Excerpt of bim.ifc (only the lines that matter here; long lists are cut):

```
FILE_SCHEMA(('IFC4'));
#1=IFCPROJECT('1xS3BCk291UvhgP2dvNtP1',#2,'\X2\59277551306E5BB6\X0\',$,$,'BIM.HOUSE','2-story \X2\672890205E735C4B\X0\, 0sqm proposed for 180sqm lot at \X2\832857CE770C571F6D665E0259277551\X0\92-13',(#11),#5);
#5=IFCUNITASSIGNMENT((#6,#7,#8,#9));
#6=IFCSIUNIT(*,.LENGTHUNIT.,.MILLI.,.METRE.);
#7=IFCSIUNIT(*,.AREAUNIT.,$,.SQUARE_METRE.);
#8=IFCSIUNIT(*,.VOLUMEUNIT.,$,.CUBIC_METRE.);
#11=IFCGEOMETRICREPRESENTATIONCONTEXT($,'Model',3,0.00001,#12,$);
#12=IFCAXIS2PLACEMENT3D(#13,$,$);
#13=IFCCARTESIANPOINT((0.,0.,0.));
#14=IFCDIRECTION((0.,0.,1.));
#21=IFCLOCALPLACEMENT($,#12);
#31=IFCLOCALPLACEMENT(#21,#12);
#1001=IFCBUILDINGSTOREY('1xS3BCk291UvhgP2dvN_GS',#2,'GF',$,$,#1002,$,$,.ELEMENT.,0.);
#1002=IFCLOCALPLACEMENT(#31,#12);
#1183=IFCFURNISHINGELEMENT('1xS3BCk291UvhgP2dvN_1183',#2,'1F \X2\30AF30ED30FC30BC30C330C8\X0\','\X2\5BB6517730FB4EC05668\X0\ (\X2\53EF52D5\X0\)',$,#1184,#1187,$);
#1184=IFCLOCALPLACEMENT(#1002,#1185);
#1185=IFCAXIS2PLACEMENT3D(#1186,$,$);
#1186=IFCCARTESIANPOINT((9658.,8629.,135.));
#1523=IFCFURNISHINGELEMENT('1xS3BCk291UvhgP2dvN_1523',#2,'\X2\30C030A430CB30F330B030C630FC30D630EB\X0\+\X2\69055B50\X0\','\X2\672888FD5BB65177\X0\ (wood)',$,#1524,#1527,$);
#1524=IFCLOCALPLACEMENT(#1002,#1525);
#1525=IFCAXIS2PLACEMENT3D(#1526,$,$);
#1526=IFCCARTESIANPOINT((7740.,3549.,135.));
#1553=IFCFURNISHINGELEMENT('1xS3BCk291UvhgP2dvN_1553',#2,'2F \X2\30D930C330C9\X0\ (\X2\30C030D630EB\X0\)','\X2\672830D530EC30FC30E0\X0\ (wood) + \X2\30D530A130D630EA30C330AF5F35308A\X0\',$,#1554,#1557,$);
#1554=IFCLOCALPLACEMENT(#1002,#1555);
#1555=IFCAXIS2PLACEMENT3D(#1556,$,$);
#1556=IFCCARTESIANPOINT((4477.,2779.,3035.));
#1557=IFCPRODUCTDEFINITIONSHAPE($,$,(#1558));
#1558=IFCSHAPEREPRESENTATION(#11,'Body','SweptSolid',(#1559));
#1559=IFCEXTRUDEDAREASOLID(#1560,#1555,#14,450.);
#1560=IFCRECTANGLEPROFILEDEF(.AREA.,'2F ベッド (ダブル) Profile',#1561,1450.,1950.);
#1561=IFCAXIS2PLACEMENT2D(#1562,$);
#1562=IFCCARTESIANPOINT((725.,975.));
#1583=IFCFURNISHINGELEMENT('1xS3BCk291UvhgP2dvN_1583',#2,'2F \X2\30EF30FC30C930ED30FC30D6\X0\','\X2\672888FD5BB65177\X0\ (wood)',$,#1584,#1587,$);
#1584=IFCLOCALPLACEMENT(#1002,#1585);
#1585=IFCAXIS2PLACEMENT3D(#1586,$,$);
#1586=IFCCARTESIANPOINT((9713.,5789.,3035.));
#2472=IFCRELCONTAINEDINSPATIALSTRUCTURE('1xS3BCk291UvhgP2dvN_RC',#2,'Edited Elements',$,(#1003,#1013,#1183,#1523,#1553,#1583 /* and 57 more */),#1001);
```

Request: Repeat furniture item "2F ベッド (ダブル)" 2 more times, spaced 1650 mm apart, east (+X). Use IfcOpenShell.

```python
import numpy as np
import ifcopenshell
import ifcopenshell.api.geometry
import ifcopenshell.api.root
import ifcopenshell.util.element
import ifcopenshell.util.placement
import ifcopenshell.util.unit

model = ifcopenshell.open("bim.ifc")
unit_scale = ifcopenshell.util.unit.calculate_unit_scale(model)


def reuse_history(source, copy):
    """copy_class also copies each property set's owner history, people and application; keep the originals."""
    for rel in copy.IsDefinedBy:
        if rel.is_a("IfcRelDefinesByProperties") and (history := rel.RelatingPropertyDefinition.OwnerHistory):
            rel.RelatingPropertyDefinition.OwnerHistory = source.OwnerHistory
            ifcopenshell.util.element.remove_deep2(model, history)


source = model.by_guid("1xS3BCk291UvhgP2dvN_1553")
base = ifcopenshell.util.placement.get_local_placement(source.ObjectPlacement)
step = np.array([1.0, 0.0, 0.0]) * 1.65 / unit_scale

for i in range(1, 3):
    copy = ifcopenshell.api.root.copy_class(model, product=source)
    copy.Representation = ifcopenshell.util.element.copy_deep(
        model, source.Representation, exclude=["IfcGeometricRepresentationContext", "IfcRepresentationMap"]
    )
    reuse_history(source, copy)
    matrix = base.copy()
    matrix[:3, 3] += i * step
    print("added at", matrix[:3, 3].round(3) + 0.0)
    ifcopenshell.api.geometry.edit_object_placement(model, product=copy, matrix=matrix, is_si=False)

model.write("bim_edited.ifc")
```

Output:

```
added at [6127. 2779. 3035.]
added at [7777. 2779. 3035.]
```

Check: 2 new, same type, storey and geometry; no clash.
